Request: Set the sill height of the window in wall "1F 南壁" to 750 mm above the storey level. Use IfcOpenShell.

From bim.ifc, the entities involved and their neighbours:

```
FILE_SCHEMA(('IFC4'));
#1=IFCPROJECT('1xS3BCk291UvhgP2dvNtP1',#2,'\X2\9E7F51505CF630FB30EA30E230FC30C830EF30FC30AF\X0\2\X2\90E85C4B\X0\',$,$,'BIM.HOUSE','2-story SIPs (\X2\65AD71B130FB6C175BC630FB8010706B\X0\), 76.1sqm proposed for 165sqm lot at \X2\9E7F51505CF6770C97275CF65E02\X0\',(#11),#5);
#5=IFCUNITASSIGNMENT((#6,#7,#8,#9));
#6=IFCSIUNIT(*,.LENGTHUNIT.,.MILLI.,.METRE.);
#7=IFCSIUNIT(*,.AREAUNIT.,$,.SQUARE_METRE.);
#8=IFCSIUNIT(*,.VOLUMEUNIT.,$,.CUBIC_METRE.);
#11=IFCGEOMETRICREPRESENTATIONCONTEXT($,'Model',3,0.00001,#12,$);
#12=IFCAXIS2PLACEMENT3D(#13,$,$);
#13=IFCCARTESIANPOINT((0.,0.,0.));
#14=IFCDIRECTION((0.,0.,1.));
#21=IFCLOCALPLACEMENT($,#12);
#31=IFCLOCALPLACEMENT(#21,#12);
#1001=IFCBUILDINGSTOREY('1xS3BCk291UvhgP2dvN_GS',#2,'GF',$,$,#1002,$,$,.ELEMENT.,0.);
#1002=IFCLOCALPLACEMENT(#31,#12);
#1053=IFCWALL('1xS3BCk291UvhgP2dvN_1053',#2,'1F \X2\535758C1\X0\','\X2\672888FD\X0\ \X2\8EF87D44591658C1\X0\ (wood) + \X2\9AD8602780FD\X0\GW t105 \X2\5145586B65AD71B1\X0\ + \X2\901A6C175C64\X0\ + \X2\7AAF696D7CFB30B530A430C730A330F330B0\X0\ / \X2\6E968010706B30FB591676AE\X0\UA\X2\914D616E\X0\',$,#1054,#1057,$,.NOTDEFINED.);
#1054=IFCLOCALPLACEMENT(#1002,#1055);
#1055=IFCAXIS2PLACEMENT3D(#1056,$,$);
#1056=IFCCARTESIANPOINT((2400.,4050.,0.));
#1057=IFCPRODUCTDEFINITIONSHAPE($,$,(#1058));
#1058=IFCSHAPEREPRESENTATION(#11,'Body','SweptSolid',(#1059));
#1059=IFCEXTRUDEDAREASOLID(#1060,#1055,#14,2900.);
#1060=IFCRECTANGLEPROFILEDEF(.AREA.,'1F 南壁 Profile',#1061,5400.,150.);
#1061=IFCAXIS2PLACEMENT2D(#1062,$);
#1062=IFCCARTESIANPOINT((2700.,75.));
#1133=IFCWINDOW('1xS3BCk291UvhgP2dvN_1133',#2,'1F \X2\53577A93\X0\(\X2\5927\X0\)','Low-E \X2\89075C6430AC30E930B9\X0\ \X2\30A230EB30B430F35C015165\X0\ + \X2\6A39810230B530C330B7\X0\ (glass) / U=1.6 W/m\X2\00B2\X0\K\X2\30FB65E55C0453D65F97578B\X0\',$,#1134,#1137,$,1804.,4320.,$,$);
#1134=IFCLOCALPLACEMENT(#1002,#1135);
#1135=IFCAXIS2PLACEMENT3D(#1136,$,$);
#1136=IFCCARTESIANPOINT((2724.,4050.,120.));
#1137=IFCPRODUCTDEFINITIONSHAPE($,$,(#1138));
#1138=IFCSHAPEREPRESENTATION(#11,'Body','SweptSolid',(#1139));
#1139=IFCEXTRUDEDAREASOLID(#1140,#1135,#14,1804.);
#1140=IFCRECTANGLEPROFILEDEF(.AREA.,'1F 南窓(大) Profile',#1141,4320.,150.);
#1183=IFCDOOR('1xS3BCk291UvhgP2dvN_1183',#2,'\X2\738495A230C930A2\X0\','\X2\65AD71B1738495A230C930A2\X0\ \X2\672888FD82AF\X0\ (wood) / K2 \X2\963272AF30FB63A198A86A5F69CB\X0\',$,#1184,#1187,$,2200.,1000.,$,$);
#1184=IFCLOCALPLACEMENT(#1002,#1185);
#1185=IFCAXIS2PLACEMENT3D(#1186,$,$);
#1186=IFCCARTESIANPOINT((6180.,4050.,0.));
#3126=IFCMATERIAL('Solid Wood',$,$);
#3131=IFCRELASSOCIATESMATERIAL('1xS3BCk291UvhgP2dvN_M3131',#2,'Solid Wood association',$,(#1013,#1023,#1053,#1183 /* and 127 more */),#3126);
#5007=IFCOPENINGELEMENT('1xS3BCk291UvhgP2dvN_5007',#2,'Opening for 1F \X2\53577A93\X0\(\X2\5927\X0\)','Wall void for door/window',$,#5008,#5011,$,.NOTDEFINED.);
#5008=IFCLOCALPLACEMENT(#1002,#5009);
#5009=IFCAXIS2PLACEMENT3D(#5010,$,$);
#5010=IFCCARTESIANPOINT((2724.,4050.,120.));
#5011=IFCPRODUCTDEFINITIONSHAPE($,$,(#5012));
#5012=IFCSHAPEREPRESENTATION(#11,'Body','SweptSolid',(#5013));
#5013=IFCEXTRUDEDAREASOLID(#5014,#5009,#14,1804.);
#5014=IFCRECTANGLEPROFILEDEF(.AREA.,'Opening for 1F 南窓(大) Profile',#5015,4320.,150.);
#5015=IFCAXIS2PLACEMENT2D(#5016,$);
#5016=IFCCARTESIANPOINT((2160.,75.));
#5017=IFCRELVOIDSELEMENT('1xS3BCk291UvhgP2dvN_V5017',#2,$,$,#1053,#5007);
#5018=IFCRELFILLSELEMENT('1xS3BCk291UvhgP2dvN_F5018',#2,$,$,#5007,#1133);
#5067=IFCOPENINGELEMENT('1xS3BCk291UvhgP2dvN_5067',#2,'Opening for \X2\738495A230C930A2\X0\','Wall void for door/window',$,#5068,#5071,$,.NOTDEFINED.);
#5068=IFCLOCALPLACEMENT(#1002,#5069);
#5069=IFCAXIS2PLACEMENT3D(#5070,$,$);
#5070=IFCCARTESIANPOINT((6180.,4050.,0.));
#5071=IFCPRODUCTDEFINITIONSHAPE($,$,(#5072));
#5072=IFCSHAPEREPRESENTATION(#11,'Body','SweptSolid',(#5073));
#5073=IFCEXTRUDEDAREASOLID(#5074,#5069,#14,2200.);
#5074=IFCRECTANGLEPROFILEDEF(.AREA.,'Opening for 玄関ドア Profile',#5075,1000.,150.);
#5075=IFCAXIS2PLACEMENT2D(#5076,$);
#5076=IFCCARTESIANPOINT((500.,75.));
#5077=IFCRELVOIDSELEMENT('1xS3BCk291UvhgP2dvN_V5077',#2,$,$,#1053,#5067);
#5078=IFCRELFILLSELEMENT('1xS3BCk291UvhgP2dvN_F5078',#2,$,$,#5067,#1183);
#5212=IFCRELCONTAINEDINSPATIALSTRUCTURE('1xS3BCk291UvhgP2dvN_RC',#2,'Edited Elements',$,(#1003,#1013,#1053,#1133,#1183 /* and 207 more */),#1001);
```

```python
import numpy as np
import ifcopenshell
import ifcopenshell.api.geometry
import ifcopenshell.geom
import ifcopenshell.util.element
import ifcopenshell.util.placement
import ifcopenshell.util.shape
import ifcopenshell.util.unit

model = ifcopenshell.open("bim.ifc")
unit_scale = ifcopenshell.util.unit.calculate_unit_scale(model)

window = model.by_guid("1xS3BCk291UvhgP2dvN_1133")
opening = window.FillsVoids[0].RelatingOpeningElement
storey = ifcopenshell.util.element.get_container(window, ifc_class="IfcBuildingStorey")
level = ifcopenshell.util.placement.get_local_placement(storey.ObjectPlacement)[2, 3]

# The opening's origin need not be at the sill, so measure its lowest point.
shape = ifcopenshell.geom.create_shape(ifcopenshell.geom.settings(), opening)
bottom = ifcopenshell.util.shape.get_shape_bottom_elevation(shape, shape.geometry) / unit_scale
dz = level + 0.75 / unit_scale - bottom

shift = np.array([0.0, 0.0, dz])
# The window is not placed relative to its opening, so move both.
for product in (opening, window):
    matrix = ifcopenshell.util.placement.get_local_placement(product.ObjectPlacement)
    matrix[:3, 3] += shift
    ifcopenshell.api.geometry.edit_object_placement(model, product=product, matrix=matrix, is_si=False)

print(f"moved by {dz * unit_scale:+.3f} m")

model.write("bim_edited.ifc")
```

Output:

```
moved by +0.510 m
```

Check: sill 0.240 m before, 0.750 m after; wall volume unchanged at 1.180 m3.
